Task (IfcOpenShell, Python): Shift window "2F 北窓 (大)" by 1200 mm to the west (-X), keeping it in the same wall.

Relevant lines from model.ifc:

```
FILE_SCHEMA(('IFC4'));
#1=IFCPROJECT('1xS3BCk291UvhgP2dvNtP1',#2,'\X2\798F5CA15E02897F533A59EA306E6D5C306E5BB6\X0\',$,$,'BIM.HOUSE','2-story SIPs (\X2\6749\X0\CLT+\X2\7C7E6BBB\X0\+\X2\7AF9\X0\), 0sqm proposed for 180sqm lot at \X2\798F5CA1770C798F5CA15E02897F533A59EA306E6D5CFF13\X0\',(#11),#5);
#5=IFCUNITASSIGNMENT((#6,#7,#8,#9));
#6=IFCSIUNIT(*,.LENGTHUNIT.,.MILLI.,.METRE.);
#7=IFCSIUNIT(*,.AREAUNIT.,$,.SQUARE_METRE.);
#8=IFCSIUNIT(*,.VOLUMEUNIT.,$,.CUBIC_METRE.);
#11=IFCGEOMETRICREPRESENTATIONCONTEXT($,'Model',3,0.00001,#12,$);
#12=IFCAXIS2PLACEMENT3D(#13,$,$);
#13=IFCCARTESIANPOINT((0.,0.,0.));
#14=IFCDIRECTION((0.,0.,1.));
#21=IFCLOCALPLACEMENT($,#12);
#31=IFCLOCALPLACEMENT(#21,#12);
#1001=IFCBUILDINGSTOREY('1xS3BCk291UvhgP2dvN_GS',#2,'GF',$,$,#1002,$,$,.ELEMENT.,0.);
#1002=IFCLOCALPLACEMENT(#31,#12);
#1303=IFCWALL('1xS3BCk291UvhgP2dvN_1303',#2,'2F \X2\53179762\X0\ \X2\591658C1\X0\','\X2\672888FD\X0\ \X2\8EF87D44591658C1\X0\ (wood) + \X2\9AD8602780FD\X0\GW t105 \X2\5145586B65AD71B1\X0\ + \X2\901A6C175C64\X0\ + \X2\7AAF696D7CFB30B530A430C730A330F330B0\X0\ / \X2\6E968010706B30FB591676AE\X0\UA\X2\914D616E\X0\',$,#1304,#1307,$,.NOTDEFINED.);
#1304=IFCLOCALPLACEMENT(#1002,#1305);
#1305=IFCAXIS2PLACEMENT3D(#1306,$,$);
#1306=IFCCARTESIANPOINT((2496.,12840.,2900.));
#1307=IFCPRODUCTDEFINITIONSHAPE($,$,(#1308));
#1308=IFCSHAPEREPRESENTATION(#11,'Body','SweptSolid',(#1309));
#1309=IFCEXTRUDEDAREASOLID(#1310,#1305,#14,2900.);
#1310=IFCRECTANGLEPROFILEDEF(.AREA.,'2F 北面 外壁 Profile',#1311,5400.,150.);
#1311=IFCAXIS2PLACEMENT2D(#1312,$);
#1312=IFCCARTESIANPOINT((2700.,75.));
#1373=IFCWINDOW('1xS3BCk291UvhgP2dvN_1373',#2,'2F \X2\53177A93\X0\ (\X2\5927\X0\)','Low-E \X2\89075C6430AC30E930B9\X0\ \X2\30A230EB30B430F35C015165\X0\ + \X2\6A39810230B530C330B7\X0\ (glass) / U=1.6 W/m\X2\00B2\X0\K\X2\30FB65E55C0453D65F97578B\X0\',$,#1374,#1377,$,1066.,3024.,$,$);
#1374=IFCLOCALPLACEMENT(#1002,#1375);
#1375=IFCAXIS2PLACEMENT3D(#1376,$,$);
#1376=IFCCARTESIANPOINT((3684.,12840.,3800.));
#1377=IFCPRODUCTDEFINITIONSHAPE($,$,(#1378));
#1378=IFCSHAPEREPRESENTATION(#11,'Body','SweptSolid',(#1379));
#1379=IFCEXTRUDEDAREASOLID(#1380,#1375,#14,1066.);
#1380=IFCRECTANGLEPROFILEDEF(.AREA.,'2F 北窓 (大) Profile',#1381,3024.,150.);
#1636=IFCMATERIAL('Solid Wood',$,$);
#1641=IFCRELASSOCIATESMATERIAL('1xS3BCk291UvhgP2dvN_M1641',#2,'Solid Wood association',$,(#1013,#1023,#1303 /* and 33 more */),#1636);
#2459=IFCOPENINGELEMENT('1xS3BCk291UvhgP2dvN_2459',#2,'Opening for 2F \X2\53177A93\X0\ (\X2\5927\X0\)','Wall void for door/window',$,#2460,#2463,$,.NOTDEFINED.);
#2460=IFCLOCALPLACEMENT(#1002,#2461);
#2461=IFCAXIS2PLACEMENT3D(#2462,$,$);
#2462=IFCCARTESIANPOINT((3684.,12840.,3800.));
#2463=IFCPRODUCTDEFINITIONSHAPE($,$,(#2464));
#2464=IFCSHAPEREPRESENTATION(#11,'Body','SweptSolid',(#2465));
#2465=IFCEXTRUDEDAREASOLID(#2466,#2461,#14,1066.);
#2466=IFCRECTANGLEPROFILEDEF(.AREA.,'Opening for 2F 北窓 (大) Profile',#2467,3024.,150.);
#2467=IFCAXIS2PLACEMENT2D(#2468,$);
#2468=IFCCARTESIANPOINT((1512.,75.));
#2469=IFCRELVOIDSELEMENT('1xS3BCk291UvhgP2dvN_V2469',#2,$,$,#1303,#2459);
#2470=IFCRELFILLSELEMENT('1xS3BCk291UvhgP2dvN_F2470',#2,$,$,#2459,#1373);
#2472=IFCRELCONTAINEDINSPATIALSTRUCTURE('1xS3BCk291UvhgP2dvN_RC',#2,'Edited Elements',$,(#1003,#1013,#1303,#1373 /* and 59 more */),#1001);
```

```python
import ifcopenshell
import ifcopenshell.api.geometry
import ifcopenshell.util.placement

model = ifcopenshell.open("model.ifc")

window = model.by_guid("1xS3BCk291UvhgP2dvN_1373")
opening = window.FillsVoids[0].RelatingOpeningElement
wall = opening.VoidsElements[0].RelatingBuildingElement

wall_matrix = ifcopenshell.util.placement.get_local_placement(wall.ObjectPlacement)
shift = wall_matrix[:3, 0] * -1200.0
before = ifcopenshell.util.placement.get_local_placement(window.ObjectPlacement)[:3, 3].copy()

# The window is not placed relative to its opening, so move both.
for product in (opening, window):
    matrix = ifcopenshell.util.placement.get_local_placement(product.ObjectPlacement)
    matrix[:3, 3] += shift
    ifcopenshell.api.geometry.edit_object_placement(model, product=product, matrix=matrix, is_si=False)

after = ifcopenshell.util.placement.get_local_placement(window.ObjectPlacement)[:3, 3]
print("window moved by", (after - before).round(3) + 0.0)

model.write("model_edited.ifc")
```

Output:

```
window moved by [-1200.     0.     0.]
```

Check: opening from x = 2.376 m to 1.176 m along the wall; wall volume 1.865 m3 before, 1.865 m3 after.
